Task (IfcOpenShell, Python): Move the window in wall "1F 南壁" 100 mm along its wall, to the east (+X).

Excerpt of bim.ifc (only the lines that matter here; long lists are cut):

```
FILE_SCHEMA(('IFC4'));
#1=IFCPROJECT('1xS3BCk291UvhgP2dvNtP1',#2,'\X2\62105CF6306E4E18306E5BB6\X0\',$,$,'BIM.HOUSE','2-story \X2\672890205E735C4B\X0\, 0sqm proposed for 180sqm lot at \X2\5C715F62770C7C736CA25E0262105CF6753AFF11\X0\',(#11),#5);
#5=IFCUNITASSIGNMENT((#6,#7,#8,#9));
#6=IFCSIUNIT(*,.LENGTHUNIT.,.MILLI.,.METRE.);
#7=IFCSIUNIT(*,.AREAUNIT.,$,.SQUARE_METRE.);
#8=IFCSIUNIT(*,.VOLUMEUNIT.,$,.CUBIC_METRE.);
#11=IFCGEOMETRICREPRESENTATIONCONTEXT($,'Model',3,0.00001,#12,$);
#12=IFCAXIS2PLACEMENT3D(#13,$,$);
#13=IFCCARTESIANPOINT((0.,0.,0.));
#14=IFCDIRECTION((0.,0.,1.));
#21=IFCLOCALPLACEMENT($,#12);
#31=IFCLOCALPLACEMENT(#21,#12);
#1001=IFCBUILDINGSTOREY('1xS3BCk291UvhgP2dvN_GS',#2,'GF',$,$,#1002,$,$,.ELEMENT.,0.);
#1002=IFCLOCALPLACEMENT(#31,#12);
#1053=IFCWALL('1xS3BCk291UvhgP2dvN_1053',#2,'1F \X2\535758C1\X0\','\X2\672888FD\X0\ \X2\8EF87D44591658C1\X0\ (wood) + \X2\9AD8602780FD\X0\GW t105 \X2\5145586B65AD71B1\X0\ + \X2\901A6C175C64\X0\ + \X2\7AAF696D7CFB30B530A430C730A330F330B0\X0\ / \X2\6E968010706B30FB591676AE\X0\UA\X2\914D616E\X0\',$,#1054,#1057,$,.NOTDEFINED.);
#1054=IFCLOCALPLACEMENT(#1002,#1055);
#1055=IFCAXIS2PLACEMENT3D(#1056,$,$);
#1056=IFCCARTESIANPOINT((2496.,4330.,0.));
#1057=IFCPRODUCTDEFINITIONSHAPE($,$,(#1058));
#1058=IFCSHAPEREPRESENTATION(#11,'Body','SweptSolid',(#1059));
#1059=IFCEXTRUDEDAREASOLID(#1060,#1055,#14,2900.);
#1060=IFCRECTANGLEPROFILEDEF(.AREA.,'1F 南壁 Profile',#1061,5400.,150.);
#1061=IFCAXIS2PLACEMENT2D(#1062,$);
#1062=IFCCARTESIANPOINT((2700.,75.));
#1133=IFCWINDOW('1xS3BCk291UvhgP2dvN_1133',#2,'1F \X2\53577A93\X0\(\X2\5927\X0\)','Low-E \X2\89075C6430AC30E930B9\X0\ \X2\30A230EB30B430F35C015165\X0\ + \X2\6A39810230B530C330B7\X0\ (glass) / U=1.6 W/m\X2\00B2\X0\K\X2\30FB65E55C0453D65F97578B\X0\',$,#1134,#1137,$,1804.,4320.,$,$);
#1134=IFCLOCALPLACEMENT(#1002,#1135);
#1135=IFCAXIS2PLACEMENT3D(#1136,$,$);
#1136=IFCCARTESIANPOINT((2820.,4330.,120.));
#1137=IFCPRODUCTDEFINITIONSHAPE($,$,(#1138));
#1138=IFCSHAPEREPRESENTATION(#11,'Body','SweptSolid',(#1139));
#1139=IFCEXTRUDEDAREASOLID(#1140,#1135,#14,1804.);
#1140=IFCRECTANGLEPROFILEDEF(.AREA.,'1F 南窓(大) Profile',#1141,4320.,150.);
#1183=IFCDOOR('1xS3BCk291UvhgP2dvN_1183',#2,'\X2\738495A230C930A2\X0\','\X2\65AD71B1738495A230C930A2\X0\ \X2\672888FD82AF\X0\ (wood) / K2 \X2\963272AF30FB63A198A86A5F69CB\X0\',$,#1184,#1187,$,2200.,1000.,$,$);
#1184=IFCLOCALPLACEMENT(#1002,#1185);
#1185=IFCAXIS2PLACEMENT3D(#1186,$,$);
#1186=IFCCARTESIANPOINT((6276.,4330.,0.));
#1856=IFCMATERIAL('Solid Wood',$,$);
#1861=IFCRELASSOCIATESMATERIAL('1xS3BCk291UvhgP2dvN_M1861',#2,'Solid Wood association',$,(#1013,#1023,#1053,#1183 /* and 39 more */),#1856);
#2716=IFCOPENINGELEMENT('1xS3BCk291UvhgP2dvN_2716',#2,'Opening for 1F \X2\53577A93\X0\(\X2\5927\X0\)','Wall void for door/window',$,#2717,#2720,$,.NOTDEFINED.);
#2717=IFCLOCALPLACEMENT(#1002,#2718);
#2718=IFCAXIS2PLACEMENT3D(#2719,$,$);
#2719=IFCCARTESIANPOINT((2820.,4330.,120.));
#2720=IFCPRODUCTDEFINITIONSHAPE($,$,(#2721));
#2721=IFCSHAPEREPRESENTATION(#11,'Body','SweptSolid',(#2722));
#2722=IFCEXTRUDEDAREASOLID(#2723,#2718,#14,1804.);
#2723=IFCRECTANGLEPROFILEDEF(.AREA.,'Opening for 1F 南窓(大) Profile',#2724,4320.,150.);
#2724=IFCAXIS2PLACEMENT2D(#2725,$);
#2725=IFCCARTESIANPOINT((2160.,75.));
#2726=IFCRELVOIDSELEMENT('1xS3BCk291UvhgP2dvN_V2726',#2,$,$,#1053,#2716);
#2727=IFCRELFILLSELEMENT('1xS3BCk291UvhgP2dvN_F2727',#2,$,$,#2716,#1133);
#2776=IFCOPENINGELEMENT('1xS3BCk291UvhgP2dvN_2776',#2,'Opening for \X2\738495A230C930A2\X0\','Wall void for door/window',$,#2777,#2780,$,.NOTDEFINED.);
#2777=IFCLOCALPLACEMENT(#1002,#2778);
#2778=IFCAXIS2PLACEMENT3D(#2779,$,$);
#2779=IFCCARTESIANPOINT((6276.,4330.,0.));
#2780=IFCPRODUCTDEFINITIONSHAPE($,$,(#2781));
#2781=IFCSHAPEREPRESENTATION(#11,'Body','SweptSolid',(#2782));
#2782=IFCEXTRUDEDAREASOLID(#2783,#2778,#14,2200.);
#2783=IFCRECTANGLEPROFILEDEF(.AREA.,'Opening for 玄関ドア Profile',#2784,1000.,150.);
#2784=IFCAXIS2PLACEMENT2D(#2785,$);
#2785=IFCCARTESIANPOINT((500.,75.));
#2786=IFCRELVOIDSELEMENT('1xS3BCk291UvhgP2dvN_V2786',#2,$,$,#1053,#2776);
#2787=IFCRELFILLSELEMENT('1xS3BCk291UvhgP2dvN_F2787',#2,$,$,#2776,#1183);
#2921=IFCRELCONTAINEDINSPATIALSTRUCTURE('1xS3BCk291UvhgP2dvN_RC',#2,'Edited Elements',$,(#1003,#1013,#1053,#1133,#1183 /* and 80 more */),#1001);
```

```python
import ifcopenshell
import ifcopenshell.api.geometry
import ifcopenshell.util.placement
import ifcopenshell.util.unit

model = ifcopenshell.open("bim.ifc")
unit_scale = ifcopenshell.util.unit.calculate_unit_scale(model)

window = model.by_guid("1xS3BCk291UvhgP2dvN_1133")
opening = window.FillsVoids[0].RelatingOpeningElement
wall = opening.VoidsElements[0].RelatingBuildingElement

wall_matrix = ifcopenshell.util.placement.get_local_placement(wall.ObjectPlacement)
shift = wall_matrix[:3, 0] * 0.1 / unit_scale
before = ifcopenshell.util.placement.get_local_placement(window.ObjectPlacement)[:3, 3].copy()

# The window is not placed relative to its opening, so move both.
for product in (opening, window):
    matrix = ifcopenshell.util.placement.get_local_placement(product.ObjectPlacement)
    matrix[:3, 3] += shift
    ifcopenshell.api.geometry.edit_object_placement(model, product=product, matrix=matrix, is_si=False)

after = ifcopenshell.util.placement.get_local_placement(window.ObjectPlacement)[:3, 3]
print("window moved by", (after - before).round(3) + 0.0)

model.write("bim_edited.ifc")
```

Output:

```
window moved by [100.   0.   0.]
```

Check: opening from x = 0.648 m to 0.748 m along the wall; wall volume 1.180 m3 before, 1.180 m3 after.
